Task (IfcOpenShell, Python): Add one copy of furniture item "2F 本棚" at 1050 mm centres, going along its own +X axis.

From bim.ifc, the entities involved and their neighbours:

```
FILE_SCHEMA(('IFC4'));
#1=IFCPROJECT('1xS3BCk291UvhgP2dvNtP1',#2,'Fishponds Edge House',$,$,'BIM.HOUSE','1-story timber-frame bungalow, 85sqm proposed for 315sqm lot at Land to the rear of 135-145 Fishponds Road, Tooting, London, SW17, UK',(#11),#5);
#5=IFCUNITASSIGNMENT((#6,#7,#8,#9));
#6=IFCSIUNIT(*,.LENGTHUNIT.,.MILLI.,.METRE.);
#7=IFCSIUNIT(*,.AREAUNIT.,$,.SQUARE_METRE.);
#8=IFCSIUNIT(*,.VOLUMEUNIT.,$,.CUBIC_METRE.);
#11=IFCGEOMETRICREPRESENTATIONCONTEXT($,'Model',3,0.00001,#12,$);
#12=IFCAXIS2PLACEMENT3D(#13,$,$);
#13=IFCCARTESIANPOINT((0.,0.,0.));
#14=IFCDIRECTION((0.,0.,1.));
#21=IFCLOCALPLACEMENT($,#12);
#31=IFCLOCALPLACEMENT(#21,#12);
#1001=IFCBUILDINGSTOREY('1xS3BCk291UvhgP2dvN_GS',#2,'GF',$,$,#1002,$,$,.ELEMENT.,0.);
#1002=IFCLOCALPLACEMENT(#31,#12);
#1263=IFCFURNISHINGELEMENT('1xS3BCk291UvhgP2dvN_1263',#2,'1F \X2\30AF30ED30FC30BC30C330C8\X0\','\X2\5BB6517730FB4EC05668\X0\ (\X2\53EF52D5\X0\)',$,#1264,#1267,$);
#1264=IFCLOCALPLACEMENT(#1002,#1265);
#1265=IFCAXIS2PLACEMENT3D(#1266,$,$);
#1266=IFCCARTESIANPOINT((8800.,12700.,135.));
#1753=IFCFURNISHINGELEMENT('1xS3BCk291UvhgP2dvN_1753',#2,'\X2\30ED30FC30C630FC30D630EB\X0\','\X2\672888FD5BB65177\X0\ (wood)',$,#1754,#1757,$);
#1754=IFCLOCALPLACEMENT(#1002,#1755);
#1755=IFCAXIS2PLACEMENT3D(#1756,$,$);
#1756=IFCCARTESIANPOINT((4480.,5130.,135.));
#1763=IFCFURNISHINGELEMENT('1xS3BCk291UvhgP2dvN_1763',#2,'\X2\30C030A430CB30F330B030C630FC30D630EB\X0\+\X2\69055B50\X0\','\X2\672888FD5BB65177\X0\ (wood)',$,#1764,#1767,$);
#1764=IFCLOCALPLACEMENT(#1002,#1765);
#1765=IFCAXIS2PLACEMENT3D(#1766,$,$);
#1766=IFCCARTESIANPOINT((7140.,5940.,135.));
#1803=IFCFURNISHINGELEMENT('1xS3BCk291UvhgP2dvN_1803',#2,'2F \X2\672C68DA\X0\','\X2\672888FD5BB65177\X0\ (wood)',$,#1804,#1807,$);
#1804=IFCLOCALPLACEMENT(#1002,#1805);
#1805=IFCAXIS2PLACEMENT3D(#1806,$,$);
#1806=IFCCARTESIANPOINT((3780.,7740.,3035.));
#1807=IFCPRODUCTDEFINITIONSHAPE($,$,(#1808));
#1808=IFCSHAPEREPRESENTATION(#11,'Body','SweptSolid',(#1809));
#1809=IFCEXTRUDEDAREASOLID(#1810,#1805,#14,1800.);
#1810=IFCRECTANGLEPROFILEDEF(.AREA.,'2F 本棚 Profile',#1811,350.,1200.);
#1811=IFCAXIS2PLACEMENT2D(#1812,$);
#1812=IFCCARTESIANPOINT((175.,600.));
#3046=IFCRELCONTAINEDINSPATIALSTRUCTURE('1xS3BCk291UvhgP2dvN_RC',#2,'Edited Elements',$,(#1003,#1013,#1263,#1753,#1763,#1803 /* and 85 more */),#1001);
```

```python
import ifcopenshell
import ifcopenshell.api.geometry
import ifcopenshell.api.root
import ifcopenshell.util.element
import ifcopenshell.util.placement

model = ifcopenshell.open("bim.ifc")


def reuse_history(source, copy):
    """copy_class also copies each property set's owner history, people and application; keep the originals."""
    for rel in copy.IsDefinedBy:
        if rel.is_a("IfcRelDefinesByProperties") and (history := rel.RelatingPropertyDefinition.OwnerHistory):
            rel.RelatingPropertyDefinition.OwnerHistory = source.OwnerHistory
            ifcopenshell.util.element.remove_deep2(model, history)


source = model.by_id(1803)
base = ifcopenshell.util.placement.get_local_placement(source.ObjectPlacement)
step = base[:3, 0] * 1050.0

for i in range(1, 2):
    copy = ifcopenshell.api.root.copy_class(model, product=source)
    copy.Representation = ifcopenshell.util.element.copy_deep(
        model, source.Representation, exclude=["IfcGeometricRepresentationContext", "IfcRepresentationMap"]
    )
    reuse_history(source, copy)
    matrix = base.copy()
    matrix[:3, 3] += i * step
    print("added at", matrix[:3, 3].round(3) + 0.0)
    ifcopenshell.api.geometry.edit_object_placement(model, product=copy, matrix=matrix, is_si=False)

model.write("bim_v2.ifc")
```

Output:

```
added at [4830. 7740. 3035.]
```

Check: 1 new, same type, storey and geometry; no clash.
